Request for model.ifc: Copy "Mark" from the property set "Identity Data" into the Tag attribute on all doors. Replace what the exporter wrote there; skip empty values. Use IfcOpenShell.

First a look at what the model holds.

```python
import ifcopenshell
import ifcopenshell.util.element

model = ifcopenshell.open("model.ifc")
print(model.schema)
doors = model.by_type("IfcDoor")
print(len(doors), "doors")
for e in doors[:8]:
    source = ifcopenshell.util.element.get_pset(e, "Identity Data", "Mark")
    target = e.Tag
    print(e.id(), repr(source), repr(target), sep=" | ")
```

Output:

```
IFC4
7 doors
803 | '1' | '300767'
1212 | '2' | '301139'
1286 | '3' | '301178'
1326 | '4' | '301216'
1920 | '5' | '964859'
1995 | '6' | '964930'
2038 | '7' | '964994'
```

```python
import ifcopenshell
import ifcopenshell.util.element

model = ifcopenshell.open("model.ifc")

count = 0
for e in model.by_type("IfcDoor"):
    value = ifcopenshell.util.element.get_pset(e, "Identity Data", "Mark")
    current = e.Tag
    if not value or not value.strip() or current == value:
        continue
    e.Tag = value
    count += 1

print(count, "doors updated")

model.write("model_edited.ifc")
```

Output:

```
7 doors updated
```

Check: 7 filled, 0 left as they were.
